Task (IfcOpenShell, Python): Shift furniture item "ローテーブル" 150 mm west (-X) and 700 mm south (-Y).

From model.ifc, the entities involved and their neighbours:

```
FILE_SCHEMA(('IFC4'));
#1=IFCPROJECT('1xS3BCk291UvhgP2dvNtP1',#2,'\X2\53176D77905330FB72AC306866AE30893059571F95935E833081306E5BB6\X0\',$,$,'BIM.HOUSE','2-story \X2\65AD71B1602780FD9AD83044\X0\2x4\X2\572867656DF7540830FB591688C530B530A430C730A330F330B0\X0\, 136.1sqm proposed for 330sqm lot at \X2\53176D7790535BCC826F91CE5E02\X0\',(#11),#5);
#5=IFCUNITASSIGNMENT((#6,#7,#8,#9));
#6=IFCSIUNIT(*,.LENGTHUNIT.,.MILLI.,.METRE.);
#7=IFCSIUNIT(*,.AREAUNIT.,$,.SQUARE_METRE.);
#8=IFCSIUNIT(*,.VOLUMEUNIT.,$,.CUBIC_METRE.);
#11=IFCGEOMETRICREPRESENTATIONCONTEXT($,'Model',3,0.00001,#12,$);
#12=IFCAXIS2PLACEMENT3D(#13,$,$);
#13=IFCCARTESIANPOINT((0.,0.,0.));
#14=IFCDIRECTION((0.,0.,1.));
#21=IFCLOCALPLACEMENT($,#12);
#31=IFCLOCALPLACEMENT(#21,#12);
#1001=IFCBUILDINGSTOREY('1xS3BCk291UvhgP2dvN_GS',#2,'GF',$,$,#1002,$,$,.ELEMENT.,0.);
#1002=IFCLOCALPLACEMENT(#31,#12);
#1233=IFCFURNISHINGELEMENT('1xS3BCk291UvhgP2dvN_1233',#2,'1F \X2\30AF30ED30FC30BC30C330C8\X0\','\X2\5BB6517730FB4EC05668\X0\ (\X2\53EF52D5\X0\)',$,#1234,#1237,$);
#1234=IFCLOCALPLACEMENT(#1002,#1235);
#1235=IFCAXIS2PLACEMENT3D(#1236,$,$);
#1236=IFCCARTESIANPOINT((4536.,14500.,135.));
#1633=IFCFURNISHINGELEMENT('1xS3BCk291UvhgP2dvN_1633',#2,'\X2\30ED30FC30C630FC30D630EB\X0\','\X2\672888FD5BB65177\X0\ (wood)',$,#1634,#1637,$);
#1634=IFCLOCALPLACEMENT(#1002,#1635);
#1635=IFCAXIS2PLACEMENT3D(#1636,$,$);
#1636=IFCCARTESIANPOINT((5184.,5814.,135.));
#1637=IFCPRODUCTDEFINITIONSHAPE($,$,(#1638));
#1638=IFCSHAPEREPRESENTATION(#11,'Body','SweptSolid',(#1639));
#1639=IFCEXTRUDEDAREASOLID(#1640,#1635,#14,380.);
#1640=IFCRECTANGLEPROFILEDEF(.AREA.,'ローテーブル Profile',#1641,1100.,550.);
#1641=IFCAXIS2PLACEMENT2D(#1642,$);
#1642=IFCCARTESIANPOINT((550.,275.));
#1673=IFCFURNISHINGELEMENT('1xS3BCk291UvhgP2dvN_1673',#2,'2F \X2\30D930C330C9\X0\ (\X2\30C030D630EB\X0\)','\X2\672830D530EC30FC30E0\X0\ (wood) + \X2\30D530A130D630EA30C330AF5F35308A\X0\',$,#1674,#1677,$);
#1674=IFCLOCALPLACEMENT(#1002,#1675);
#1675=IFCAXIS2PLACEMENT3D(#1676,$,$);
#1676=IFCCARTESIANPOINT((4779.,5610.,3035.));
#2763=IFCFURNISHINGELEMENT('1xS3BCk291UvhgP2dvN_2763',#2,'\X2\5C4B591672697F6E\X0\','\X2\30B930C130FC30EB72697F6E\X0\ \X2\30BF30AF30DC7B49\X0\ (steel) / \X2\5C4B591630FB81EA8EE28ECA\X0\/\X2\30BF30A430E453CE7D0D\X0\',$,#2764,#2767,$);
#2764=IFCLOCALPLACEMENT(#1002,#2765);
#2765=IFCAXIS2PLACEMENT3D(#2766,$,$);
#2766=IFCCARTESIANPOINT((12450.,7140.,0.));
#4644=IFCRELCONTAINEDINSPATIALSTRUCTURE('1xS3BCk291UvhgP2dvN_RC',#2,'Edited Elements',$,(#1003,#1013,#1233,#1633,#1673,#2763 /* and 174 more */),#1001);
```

```python
import ifcopenshell
import ifcopenshell.api.geometry
import ifcopenshell.util.placement
import ifcopenshell.util.unit

model = ifcopenshell.open("model.ifc")
unit_scale = ifcopenshell.util.unit.calculate_unit_scale(model)

item = model.by_id(1633)
matrix = ifcopenshell.util.placement.get_local_placement(item.ObjectPlacement)
matrix[0, 3] -= 0.15 / unit_scale
matrix[1, 3] -= 0.7 / unit_scale
ifcopenshell.api.geometry.edit_object_placement(model, product=item, matrix=matrix, is_si=False)

print(ifcopenshell.util.placement.get_local_placement(item.ObjectPlacement).round(3) + 0.0)

model.write("model_rev.ifc")
```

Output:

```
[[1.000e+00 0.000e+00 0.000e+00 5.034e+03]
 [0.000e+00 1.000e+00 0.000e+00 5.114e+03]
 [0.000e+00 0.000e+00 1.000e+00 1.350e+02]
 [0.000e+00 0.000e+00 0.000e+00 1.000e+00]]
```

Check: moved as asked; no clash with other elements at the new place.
